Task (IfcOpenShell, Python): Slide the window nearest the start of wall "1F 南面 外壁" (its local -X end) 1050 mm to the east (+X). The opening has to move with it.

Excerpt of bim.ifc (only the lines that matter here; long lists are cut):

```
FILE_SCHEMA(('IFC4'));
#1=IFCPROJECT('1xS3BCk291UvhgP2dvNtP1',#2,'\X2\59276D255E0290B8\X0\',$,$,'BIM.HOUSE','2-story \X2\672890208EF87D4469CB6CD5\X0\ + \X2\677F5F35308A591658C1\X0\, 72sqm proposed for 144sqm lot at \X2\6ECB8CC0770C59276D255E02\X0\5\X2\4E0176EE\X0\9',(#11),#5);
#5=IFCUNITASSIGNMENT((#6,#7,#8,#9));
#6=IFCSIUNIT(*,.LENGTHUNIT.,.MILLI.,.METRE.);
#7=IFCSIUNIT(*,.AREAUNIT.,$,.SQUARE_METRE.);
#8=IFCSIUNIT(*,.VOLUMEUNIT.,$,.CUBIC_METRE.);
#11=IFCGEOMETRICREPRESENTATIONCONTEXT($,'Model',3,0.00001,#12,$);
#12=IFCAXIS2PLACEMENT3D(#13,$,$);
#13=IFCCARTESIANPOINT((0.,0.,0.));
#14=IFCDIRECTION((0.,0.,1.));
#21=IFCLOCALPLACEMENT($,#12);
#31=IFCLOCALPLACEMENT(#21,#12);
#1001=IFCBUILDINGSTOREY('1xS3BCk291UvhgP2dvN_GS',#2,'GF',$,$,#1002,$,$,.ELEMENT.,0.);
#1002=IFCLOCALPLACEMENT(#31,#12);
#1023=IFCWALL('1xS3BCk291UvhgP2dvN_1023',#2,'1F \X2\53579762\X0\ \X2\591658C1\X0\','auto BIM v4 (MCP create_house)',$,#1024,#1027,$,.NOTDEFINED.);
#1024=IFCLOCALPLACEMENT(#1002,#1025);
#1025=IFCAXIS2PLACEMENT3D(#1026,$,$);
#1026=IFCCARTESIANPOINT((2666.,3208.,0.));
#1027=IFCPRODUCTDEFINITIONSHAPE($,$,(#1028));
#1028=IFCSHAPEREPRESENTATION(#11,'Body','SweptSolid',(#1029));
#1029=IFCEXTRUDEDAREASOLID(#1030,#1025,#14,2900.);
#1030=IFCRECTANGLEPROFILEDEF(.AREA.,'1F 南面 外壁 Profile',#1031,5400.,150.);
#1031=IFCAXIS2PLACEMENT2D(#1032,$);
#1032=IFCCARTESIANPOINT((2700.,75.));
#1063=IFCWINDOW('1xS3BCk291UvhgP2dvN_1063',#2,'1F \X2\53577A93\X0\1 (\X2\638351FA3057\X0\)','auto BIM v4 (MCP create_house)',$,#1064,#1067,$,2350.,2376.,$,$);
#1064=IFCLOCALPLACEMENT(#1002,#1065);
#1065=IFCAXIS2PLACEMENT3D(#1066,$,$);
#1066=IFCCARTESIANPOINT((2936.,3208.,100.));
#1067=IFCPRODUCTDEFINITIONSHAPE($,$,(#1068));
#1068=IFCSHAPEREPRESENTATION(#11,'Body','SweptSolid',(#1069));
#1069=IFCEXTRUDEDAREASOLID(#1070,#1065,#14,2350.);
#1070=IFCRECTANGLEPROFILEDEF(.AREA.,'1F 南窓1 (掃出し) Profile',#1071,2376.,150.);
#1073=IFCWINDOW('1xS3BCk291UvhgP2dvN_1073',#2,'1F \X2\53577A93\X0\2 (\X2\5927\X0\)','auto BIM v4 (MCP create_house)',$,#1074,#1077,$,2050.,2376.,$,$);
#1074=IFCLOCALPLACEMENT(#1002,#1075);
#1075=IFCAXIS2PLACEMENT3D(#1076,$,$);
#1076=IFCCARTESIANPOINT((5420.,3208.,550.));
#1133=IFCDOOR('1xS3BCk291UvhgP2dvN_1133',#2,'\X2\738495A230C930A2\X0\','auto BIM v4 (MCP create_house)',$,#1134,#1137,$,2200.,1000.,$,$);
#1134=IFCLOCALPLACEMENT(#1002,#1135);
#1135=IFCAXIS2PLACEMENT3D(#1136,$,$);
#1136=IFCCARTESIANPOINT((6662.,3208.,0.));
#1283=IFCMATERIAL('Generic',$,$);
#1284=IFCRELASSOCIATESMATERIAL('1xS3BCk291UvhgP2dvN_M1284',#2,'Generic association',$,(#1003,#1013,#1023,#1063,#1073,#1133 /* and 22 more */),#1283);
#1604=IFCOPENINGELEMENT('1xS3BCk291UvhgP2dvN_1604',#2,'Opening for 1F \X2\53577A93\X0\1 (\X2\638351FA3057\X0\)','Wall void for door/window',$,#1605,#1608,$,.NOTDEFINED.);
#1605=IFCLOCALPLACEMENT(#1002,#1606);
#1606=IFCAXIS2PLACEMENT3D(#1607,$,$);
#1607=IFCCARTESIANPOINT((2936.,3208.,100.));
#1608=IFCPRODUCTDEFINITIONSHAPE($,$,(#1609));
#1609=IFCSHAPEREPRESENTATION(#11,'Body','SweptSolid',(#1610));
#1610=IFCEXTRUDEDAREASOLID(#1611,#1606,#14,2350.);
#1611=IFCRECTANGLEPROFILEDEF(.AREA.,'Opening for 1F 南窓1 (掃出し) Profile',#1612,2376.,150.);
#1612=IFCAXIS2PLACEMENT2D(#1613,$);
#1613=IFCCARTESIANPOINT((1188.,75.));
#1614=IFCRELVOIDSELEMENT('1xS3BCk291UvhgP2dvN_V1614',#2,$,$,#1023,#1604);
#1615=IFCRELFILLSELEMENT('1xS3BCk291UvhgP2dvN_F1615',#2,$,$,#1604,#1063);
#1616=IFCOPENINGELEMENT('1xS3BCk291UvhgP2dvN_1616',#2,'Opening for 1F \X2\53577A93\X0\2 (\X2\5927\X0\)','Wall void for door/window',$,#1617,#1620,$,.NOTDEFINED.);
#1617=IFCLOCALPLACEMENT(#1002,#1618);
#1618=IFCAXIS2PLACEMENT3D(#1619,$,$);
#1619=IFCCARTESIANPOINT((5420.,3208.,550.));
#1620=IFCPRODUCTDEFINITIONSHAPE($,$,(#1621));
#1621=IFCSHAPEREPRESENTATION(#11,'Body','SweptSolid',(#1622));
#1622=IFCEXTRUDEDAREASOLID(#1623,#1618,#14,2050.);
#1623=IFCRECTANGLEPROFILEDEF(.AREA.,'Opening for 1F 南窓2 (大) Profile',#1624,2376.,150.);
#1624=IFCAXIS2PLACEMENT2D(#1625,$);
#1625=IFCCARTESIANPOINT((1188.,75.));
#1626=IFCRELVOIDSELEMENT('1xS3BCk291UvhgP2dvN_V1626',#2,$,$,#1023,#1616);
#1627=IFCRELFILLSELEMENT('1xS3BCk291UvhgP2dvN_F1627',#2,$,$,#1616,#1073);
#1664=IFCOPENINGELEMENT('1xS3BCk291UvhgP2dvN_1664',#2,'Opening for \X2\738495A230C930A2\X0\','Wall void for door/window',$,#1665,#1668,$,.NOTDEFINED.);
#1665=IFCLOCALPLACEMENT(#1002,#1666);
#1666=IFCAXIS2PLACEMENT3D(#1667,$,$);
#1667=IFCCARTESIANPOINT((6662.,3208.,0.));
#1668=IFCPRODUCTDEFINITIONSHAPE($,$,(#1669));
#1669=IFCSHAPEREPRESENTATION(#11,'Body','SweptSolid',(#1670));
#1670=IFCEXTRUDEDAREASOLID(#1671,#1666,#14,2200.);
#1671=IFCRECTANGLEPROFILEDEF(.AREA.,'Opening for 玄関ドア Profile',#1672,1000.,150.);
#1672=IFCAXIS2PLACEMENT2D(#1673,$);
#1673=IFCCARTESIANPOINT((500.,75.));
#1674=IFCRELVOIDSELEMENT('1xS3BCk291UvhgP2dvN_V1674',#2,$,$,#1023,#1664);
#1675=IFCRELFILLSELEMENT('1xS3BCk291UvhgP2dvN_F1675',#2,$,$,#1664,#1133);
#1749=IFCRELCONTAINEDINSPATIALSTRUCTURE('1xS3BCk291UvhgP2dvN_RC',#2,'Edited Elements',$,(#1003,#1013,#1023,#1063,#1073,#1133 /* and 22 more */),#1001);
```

```python
import ifcopenshell
import ifcopenshell.api.geometry
import ifcopenshell.util.placement
import ifcopenshell.util.unit

model = ifcopenshell.open("bim.ifc")
unit_scale = ifcopenshell.util.unit.calculate_unit_scale(model)

window = model.by_guid("1xS3BCk291UvhgP2dvN_1063")
opening = window.FillsVoids[0].RelatingOpeningElement
wall = opening.VoidsElements[0].RelatingBuildingElement

wall_matrix = ifcopenshell.util.placement.get_local_placement(wall.ObjectPlacement)
shift = wall_matrix[:3, 0] * 1.05 / unit_scale
before = ifcopenshell.util.placement.get_local_placement(window.ObjectPlacement)[:3, 3].copy()

# The window is not placed relative to its opening, so move both.
for product in (opening, window):
    matrix = ifcopenshell.util.placement.get_local_placement(product.ObjectPlacement)
    matrix[:3, 3] += shift
    ifcopenshell.api.geometry.edit_object_placement(model, product=product, matrix=matrix, is_si=False)

after = ifcopenshell.util.placement.get_local_placement(window.ObjectPlacement)[:3, 3]
print("window moved by", (after - before).round(3) + 0.0)

model.write("bim_updated.ifc")
```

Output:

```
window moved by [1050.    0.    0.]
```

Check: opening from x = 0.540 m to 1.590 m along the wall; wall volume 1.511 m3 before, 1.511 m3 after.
